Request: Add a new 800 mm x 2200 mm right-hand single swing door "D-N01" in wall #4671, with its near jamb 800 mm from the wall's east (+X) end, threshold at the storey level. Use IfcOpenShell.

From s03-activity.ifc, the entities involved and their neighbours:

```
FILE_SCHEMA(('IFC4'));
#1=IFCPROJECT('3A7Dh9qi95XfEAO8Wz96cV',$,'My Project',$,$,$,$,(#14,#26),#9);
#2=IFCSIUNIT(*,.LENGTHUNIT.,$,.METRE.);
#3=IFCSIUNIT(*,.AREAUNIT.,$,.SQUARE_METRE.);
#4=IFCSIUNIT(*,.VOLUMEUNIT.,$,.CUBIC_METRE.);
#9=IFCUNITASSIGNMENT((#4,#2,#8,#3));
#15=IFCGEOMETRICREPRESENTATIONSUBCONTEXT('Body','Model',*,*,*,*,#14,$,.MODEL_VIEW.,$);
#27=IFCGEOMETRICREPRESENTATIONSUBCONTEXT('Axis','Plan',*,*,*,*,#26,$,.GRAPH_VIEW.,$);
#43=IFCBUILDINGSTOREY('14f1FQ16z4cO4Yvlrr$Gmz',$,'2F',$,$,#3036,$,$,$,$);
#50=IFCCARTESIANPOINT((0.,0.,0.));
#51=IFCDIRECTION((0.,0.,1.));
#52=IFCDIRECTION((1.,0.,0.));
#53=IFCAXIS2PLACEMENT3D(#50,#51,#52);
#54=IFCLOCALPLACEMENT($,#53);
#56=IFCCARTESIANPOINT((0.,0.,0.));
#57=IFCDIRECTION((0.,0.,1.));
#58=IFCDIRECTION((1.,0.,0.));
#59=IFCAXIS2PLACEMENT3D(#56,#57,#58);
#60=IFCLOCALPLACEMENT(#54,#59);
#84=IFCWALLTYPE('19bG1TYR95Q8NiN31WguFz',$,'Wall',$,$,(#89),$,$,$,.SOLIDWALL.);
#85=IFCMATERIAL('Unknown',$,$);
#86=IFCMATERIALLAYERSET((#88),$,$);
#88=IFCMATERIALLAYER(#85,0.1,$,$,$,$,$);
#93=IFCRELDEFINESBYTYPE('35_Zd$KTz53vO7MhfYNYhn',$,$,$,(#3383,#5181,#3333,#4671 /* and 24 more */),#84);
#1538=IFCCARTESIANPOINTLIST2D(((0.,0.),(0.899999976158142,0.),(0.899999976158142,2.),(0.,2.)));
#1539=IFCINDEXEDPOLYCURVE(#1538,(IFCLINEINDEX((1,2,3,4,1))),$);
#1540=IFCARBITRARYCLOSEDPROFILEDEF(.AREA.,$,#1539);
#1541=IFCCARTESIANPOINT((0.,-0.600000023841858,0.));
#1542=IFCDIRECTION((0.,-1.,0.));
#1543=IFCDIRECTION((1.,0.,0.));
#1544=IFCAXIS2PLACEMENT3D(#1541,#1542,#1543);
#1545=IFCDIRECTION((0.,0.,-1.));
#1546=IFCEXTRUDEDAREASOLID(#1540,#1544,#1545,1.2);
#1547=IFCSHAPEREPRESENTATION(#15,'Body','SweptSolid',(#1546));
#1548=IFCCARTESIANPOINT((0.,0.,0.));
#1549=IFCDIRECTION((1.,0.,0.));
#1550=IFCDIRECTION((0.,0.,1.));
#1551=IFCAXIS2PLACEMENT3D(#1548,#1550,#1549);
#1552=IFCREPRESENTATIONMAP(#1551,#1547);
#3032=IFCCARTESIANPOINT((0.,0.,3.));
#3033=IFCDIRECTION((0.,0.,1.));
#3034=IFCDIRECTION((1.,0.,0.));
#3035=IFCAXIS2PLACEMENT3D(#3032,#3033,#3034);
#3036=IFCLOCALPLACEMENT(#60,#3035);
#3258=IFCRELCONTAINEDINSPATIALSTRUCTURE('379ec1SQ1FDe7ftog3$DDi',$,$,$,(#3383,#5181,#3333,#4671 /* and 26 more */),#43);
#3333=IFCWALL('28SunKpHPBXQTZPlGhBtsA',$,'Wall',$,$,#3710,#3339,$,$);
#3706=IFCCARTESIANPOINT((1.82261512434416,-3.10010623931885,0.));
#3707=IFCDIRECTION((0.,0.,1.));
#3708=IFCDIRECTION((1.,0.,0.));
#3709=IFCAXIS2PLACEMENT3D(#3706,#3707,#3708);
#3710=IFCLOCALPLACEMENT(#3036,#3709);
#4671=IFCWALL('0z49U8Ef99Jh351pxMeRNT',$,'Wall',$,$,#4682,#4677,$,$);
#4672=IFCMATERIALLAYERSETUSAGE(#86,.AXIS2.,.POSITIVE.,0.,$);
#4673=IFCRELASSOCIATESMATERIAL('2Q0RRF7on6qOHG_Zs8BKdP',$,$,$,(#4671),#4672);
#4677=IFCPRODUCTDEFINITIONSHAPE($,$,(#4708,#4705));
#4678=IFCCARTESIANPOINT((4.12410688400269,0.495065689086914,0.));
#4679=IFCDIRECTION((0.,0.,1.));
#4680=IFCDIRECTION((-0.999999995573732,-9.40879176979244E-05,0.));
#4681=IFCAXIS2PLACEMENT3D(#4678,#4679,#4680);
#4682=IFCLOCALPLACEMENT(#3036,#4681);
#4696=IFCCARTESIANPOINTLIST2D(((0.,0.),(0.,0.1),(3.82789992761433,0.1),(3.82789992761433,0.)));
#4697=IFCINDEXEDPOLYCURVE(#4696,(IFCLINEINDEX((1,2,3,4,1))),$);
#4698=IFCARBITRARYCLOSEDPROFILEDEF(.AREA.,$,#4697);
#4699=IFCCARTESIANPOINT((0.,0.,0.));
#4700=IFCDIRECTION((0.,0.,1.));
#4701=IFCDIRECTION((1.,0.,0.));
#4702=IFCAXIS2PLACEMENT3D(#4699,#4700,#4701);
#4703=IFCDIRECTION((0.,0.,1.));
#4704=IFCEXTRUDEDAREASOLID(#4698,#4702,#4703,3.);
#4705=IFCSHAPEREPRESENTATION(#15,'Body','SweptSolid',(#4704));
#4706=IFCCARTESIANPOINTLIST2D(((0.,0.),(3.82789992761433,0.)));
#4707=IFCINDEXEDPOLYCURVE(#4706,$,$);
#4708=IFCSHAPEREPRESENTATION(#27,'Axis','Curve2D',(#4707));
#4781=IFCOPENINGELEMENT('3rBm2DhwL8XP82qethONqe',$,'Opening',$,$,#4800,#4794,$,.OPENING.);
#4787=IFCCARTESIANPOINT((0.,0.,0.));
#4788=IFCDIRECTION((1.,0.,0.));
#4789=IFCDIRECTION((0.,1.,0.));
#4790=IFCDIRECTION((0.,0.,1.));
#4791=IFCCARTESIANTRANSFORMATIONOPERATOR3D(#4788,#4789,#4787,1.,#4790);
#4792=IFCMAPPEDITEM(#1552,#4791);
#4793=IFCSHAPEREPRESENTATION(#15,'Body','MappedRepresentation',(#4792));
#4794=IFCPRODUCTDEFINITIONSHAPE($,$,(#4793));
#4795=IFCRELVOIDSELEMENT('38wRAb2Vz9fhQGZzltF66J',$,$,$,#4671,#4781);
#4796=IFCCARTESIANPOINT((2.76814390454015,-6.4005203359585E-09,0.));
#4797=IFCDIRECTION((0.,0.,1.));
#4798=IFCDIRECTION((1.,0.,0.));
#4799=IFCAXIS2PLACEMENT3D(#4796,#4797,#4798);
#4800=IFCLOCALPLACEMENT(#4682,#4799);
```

```python
import numpy as np
import ifcopenshell
import ifcopenshell.api.feature
import ifcopenshell.api.geometry
import ifcopenshell.api.root
import ifcopenshell.api.spatial
import ifcopenshell.geom
import ifcopenshell.util.element
import ifcopenshell.util.placement
import ifcopenshell.util.representation
import ifcopenshell.util.shape
import ifcopenshell.util.unit

model = ifcopenshell.open("s03-activity.ifc")
unit_scale = ifcopenshell.util.unit.calculate_unit_scale(model)
settings = ifcopenshell.geom.settings()


def volume(element):
    """Net volume in cubic metres, openings subtracted."""
    shape = ifcopenshell.geom.create_shape(settings, element)
    return ifcopenshell.util.shape.get_volume(shape.geometry)


wall = model.by_guid("0z49U8Ef99Jh351pxMeRNT")
storey = ifcopenshell.util.element.get_container(wall, ifc_class="IfcBuildingStorey")
context = ifcopenshell.util.representation.get_context(model, "Model", "Body", "MODEL_VIEW")
before = volume(wall)

width, height, from_end, sill = 0.8, 2.2, 0.8, 0.0  # metres

# The wall runs along its own X axis, and the end named is its -X end.
wall_shape = ifcopenshell.geom.create_shape(settings, wall)
x, y, z = ifcopenshell.util.shape.get_vertices(wall_shape.geometry).T
start = x.min() + from_end
face, thickness = float(y.min()), float(y.max() - y.min())
wall_matrix = ifcopenshell.util.placement.get_local_placement(wall.ObjectPlacement)
level = ifcopenshell.util.placement.get_local_placement(storey.ObjectPlacement)[2, 3]


def in_wall(x, y):
    """Placement at x, y metres in the wall's axes, at sill height."""
    matrix = wall_matrix.copy()
    matrix[:, 3] = wall_matrix @ np.array([x / unit_scale, y / unit_scale, 0.0, 1.0])
    matrix[2, 3] = level + sill / unit_scale
    return matrix


# Opening: a box that overshoots both wall faces by 50 mm.
opening = ifcopenshell.api.root.create_entity(model, ifc_class="IfcOpeningElement", predefined_type="OPENING")
box = ifcopenshell.api.geometry.add_wall_representation(
    model, context=context, length=width, height=height, thickness=thickness + 0.1
)
ifcopenshell.api.geometry.assign_representation(model, product=opening, representation=box)
ifcopenshell.api.geometry.edit_object_placement(model, product=opening, matrix=in_wall(start, face - 0.05), is_si=False)
ifcopenshell.api.feature.add_feature(model, feature=opening, element=wall)

door = ifcopenshell.api.root.create_entity(model, ifc_class="IfcDoor", name="D-N01", predefined_type="DOOR")
door.OverallWidth, door.OverallHeight = width / unit_scale, height / unit_scale
door.OperationType = "SINGLE_SWING_RIGHT"
body = ifcopenshell.api.geometry.add_door_representation(
    model,
    context=context,
    overall_width=door.OverallWidth,
    overall_height=door.OverallHeight,
    operation_type="SINGLE_SWING_RIGHT",
    lining_properties={"LiningDepth": thickness / unit_scale, "ThresholdDepth": thickness / unit_scale},
)
ifcopenshell.api.geometry.assign_representation(model, product=door, representation=body)
ifcopenshell.api.spatial.assign_container(model, products=[door], relating_structure=storey)
ifcopenshell.api.feature.add_filling(model, opening=opening, element=door)

# The lining spans the wall, so the door starts at the wall face.
ifcopenshell.api.geometry.edit_object_placement(model, product=door, matrix=in_wall(start, face), is_si=False)

after = volume(wall)

print(f"wall volume {before:.3f} -> {after:.3f} m3")

model.write("s03-activity_updated.ifc")
```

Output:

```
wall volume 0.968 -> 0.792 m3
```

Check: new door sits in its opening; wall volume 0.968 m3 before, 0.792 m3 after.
